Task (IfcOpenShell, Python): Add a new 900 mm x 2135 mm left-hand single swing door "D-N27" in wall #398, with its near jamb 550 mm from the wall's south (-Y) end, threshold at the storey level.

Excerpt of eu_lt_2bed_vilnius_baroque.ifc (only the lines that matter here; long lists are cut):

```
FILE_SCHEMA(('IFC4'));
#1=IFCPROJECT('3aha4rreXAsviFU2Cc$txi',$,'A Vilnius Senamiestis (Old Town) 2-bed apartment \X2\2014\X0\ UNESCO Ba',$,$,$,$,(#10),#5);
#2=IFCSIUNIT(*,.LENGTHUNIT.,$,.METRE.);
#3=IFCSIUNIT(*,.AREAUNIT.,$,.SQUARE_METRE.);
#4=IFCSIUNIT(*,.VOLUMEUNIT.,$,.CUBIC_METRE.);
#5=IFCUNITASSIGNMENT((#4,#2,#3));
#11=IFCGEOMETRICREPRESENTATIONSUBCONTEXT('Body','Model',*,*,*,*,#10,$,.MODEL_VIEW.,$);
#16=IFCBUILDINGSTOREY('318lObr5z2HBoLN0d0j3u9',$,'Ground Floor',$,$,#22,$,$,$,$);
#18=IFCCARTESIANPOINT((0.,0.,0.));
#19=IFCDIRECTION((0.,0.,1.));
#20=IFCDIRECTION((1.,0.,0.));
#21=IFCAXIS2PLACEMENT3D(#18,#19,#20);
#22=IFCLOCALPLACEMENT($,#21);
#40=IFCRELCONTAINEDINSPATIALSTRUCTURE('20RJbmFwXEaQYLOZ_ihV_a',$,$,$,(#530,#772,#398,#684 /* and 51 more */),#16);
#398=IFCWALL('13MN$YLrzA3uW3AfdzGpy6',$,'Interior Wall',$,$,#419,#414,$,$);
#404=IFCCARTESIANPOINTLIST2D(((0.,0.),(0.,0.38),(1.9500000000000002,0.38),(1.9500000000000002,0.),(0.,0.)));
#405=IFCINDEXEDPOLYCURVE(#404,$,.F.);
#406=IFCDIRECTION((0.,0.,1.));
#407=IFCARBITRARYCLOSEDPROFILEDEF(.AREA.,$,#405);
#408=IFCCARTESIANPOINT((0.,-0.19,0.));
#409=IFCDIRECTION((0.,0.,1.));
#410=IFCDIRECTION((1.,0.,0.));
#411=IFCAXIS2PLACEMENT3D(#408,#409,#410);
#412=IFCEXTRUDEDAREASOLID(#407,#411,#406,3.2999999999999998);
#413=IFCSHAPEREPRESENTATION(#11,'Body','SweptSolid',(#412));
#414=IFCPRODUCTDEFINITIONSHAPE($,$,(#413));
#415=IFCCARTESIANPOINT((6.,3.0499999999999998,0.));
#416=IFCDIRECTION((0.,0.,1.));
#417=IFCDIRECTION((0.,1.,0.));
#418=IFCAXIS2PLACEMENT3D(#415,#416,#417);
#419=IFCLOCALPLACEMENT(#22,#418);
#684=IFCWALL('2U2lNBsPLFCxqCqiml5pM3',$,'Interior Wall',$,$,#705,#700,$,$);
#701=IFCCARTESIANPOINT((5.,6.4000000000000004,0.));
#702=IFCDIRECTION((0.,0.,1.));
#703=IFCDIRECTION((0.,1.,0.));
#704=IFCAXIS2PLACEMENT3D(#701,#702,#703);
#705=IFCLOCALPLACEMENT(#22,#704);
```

```python
import numpy as np
import ifcopenshell
import ifcopenshell.api.feature
import ifcopenshell.api.geometry
import ifcopenshell.api.root
import ifcopenshell.api.spatial
import ifcopenshell.geom
import ifcopenshell.util.element
import ifcopenshell.util.placement
import ifcopenshell.util.representation
import ifcopenshell.util.shape
import ifcopenshell.util.unit

model = ifcopenshell.open("eu_lt_2bed_vilnius_baroque.ifc")
unit_scale = ifcopenshell.util.unit.calculate_unit_scale(model)
settings = ifcopenshell.geom.settings()


def volume(element):
    """Net volume in cubic metres, openings subtracted."""
    shape = ifcopenshell.geom.create_shape(settings, element)
    return ifcopenshell.util.shape.get_volume(shape.geometry)


wall = model.by_id(398)
storey = ifcopenshell.util.element.get_container(wall, ifc_class="IfcBuildingStorey")
context = ifcopenshell.util.representation.get_context(model, "Model", "Body", "MODEL_VIEW")
before = volume(wall)

width, height, from_end, sill = 0.9, 2.135, 0.55, 0.0  # metres

# The wall runs along its own X axis, and the end named is its -X end.
wall_shape = ifcopenshell.geom.create_shape(settings, wall)
x, y, z = ifcopenshell.util.shape.get_vertices(wall_shape.geometry).T
start = x.min() + from_end
face, thickness = float(y.min()), float(y.max() - y.min())
wall_matrix = ifcopenshell.util.placement.get_local_placement(wall.ObjectPlacement)
level = ifcopenshell.util.placement.get_local_placement(storey.ObjectPlacement)[2, 3]


def in_wall(x, y):
    """Placement at x, y metres in the wall's axes, at sill height."""
    matrix = wall_matrix.copy()
    matrix[:, 3] = wall_matrix @ np.array([x / unit_scale, y / unit_scale, 0.0, 1.0])
    matrix[2, 3] = level + sill / unit_scale
    return matrix


# Opening: a box that overshoots both wall faces by 50 mm.
opening = ifcopenshell.api.root.create_entity(model, ifc_class="IfcOpeningElement", predefined_type="OPENING")
box = ifcopenshell.api.geometry.add_wall_representation(
    model, context=context, length=width, height=height, thickness=thickness + 0.1
)
ifcopenshell.api.geometry.assign_representation(model, product=opening, representation=box)
ifcopenshell.api.geometry.edit_object_placement(model, product=opening, matrix=in_wall(start, face - 0.05), is_si=False)
ifcopenshell.api.feature.add_feature(model, feature=opening, element=wall)

door = ifcopenshell.api.root.create_entity(model, ifc_class="IfcDoor", name="D-N27", predefined_type="DOOR")
door.OverallWidth, door.OverallHeight = width / unit_scale, height / unit_scale
door.OperationType = "SINGLE_SWING_LEFT"
body = ifcopenshell.api.geometry.add_door_representation(
    model,
    context=context,
    overall_width=door.OverallWidth,
    overall_height=door.OverallHeight,
    operation_type="SINGLE_SWING_LEFT",
    lining_properties={"LiningDepth": thickness / unit_scale, "ThresholdDepth": thickness / unit_scale},
)
ifcopenshell.api.geometry.assign_representation(model, product=door, representation=body)
ifcopenshell.api.spatial.assign_container(model, products=[door], relating_structure=storey)
ifcopenshell.api.feature.add_filling(model, opening=opening, element=door)

# The lining spans the wall, so the door starts at the wall face.
ifcopenshell.api.geometry.edit_object_placement(model, product=door, matrix=in_wall(start, face), is_si=False)

after = volume(wall)

print(f"wall volume {before:.3f} -> {after:.3f} m3")

model.write("eu_lt_2bed_vilnius_baroque-out.ifc")
```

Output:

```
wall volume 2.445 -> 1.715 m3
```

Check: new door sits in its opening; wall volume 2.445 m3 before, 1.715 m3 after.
